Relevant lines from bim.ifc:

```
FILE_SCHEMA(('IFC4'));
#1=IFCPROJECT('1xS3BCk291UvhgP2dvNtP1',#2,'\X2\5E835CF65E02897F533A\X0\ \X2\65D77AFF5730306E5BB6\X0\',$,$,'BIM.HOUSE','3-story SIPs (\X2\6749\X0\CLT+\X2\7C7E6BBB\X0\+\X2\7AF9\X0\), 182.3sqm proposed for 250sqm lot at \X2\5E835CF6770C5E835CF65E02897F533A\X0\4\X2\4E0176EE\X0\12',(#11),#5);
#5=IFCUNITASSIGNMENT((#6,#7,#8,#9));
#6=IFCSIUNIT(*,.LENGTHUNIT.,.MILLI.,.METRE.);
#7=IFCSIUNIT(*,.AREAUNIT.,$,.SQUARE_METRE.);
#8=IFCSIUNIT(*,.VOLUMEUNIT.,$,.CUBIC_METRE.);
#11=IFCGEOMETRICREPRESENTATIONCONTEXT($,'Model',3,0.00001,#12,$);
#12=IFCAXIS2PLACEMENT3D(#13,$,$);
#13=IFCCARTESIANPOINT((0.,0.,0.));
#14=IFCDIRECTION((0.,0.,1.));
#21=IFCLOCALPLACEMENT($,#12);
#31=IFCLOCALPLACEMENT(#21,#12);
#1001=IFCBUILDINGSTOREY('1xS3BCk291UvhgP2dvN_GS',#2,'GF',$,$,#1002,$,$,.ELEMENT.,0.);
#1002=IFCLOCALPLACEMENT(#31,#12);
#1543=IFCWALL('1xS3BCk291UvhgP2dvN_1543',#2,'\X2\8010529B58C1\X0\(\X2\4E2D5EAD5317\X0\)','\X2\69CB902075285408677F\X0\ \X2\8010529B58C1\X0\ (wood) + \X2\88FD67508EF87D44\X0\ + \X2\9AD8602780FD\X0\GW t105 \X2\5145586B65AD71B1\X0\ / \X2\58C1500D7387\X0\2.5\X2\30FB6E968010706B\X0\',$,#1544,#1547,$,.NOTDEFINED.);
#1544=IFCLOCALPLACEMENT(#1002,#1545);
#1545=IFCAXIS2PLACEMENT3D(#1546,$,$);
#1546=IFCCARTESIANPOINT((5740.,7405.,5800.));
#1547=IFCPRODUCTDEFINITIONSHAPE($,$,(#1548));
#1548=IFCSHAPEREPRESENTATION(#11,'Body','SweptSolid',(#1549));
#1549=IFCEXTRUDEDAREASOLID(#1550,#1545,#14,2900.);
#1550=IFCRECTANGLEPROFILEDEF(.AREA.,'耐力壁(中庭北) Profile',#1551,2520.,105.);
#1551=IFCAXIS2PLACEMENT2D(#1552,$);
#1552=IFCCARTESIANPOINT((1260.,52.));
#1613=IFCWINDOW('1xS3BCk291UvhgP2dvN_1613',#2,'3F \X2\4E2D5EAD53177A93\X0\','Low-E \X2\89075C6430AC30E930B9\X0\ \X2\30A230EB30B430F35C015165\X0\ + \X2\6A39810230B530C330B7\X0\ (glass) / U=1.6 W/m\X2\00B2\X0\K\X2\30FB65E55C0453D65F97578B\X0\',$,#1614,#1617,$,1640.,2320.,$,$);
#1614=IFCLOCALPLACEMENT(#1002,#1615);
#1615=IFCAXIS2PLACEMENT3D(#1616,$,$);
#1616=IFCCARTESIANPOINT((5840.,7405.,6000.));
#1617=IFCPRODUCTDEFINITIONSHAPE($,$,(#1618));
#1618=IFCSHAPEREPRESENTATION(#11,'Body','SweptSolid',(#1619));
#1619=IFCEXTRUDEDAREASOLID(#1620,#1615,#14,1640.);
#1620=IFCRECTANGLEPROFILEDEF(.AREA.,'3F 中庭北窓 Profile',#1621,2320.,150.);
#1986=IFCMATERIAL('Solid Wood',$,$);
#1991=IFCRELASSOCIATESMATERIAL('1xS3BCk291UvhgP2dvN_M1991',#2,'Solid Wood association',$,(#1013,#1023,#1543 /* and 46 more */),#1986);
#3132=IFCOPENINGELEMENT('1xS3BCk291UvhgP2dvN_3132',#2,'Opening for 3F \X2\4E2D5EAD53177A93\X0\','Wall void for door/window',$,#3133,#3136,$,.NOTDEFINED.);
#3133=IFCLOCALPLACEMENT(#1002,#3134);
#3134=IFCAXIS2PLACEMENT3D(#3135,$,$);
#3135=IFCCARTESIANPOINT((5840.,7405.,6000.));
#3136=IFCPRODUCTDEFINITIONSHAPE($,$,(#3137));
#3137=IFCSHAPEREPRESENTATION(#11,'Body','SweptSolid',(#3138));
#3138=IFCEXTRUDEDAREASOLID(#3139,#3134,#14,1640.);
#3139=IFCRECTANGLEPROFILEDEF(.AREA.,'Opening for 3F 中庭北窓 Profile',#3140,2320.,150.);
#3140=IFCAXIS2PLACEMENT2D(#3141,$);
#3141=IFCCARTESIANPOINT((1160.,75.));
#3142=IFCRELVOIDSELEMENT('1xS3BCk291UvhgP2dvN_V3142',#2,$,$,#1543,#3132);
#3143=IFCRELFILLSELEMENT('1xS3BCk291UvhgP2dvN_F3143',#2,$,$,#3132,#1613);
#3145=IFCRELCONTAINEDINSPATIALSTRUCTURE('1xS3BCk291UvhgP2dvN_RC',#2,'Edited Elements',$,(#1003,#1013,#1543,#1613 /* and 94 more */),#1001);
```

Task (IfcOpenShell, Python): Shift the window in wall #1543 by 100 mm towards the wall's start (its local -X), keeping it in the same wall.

```python
import ifcopenshell
import ifcopenshell.api.geometry
import ifcopenshell.util.placement

model = ifcopenshell.open("bim.ifc")

window = model.by_guid("1xS3BCk291UvhgP2dvN_1613")
opening = window.FillsVoids[0].RelatingOpeningElement
wall = opening.VoidsElements[0].RelatingBuildingElement

wall_matrix = ifcopenshell.util.placement.get_local_placement(wall.ObjectPlacement)
shift = wall_matrix[:3, 0] * -100.0
before = ifcopenshell.util.placement.get_local_placement(window.ObjectPlacement)[:3, 3].copy()

# The window is not placed relative to its opening, so move both.
for product in (opening, window):
    matrix = ifcopenshell.util.placement.get_local_placement(product.ObjectPlacement)
    matrix[:3, 3] += shift
    ifcopenshell.api.geometry.edit_object_placement(model, product=product, matrix=matrix, is_si=False)

after = ifcopenshell.util.placement.get_local_placement(window.ObjectPlacement)[:3, 3]
print("window moved by", (after - before).round(3) + 0.0)

model.write("bim_edited.ifc")
```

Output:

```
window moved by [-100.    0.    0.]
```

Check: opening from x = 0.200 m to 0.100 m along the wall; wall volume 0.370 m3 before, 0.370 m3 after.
